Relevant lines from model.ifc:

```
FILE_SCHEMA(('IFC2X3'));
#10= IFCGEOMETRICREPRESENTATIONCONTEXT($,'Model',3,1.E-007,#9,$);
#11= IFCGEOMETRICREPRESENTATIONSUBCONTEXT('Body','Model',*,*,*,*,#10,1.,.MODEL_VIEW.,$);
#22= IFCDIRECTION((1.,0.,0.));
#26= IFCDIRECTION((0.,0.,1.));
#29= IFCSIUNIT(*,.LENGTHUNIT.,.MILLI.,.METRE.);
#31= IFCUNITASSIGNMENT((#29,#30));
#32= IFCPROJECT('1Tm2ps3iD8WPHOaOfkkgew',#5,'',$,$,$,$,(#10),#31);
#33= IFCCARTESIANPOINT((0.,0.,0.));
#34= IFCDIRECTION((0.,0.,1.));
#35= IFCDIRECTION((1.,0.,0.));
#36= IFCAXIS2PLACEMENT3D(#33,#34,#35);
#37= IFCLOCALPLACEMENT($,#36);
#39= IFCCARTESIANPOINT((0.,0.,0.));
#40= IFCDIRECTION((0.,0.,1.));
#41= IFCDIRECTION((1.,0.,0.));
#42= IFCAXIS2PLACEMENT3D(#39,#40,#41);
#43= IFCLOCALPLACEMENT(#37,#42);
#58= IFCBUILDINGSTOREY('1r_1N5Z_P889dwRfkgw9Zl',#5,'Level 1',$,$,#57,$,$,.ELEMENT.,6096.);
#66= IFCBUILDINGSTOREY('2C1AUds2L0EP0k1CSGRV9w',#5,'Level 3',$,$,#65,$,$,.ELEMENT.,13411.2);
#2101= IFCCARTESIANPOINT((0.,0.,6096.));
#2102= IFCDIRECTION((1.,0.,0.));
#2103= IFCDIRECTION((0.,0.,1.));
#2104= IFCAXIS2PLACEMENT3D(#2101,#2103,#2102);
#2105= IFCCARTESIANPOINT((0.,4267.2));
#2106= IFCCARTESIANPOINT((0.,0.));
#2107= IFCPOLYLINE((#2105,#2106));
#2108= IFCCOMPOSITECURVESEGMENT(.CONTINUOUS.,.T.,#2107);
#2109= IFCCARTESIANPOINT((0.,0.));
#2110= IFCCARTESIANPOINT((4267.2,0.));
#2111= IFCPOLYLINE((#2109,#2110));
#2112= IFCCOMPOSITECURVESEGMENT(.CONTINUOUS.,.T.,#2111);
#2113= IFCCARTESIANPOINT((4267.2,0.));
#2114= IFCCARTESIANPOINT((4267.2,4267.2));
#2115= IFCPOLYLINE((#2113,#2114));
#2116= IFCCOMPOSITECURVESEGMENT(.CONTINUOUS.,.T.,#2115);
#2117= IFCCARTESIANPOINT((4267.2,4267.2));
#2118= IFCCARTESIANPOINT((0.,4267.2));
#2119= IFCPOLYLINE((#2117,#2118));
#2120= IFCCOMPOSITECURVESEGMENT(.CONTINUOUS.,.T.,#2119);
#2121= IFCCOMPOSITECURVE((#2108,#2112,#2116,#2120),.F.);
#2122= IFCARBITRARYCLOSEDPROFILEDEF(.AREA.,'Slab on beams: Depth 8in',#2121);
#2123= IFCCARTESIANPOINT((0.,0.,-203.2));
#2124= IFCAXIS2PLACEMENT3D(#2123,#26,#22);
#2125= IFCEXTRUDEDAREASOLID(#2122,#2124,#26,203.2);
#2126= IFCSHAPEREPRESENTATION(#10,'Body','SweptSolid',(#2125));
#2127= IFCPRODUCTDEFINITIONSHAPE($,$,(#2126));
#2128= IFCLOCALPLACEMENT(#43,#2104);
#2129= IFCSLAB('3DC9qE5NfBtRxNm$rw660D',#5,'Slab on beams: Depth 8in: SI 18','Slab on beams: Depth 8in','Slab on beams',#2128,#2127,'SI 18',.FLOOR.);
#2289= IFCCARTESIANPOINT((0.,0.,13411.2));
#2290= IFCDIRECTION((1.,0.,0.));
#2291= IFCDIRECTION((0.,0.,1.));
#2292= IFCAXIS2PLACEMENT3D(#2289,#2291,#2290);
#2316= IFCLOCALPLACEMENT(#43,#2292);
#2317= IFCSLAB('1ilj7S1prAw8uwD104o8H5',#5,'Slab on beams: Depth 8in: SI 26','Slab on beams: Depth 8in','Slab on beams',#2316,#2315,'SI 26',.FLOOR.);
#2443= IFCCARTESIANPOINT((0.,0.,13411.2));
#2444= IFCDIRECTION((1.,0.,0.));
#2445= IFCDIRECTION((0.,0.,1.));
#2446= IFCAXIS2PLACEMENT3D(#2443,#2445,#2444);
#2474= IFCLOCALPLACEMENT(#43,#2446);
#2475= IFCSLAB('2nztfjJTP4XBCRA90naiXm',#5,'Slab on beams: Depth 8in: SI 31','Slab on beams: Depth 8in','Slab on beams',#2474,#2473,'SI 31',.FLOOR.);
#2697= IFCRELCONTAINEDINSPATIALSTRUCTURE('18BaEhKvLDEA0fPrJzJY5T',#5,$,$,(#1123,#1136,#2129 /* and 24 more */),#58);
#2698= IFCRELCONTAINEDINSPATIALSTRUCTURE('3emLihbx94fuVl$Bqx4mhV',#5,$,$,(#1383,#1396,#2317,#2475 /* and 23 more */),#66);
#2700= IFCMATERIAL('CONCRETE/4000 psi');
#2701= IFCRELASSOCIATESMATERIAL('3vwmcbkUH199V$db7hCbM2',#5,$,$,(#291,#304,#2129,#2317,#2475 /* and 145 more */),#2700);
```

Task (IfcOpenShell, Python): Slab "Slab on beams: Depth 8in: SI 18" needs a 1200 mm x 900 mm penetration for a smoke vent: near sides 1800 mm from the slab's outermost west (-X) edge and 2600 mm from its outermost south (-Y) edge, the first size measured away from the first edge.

```python
import numpy as np
import ifcopenshell
import ifcopenshell.api.feature
import ifcopenshell.api.geometry
import ifcopenshell.api.root
import ifcopenshell.geom
import ifcopenshell.util.placement
import ifcopenshell.util.representation
import ifcopenshell.util.shape
import ifcopenshell.util.unit

model = ifcopenshell.open("model.ifc")
unit_scale = ifcopenshell.util.unit.calculate_unit_scale(model)
settings = ifcopenshell.geom.settings()


def volume(element):
    """Net volume in cubic metres, openings subtracted."""
    shape = ifcopenshell.geom.create_shape(settings, element)
    return ifcopenshell.util.shape.get_volume(shape.geometry)


slab = model.by_id(2129)
before = volume(slab)

# Extent in the slab's own axes, in metres. The edges named are its -X and -Y sides.
slab_shape = ifcopenshell.geom.create_shape(settings, slab)
vertices = ifcopenshell.util.shape.get_vertices(slab_shape.geometry)
x_min, y_min, bottom = vertices.min(axis=0)
top = vertices[:, 2].max()

opening = ifcopenshell.api.root.create_entity(model, ifc_class="IfcOpeningElement", name="Smoke vent opening")
context = ifcopenshell.util.representation.get_context(model, "Model", "Body", "MODEL_VIEW")
width, depth = 1.2, 0.9
outline = [(0.0, 0.0), (width, 0.0), (width, depth), (0.0, depth), (0.0, 0.0)]
# Overshoot both faces by 50 mm so the cut is clean.
shape = ifcopenshell.api.geometry.add_slab_representation(
    model, context=context, depth=top - bottom + 0.1, polyline=outline
)
ifcopenshell.api.geometry.assign_representation(model, product=opening, representation=shape)

matrix = ifcopenshell.util.placement.get_local_placement(slab.ObjectPlacement)
matrix[:, 3] = matrix @ np.append(np.array([x_min + 1.8, y_min + 2.6, bottom - 0.05]) / unit_scale, 1.0)
ifcopenshell.api.geometry.edit_object_placement(model, product=opening, matrix=matrix, is_si=False)
ifcopenshell.api.feature.add_feature(model, feature=opening, element=slab)

after = volume(slab)

print(f"slab volume {before:.3f} -> {after:.3f} m3")

model.write("model-out.ifc")
```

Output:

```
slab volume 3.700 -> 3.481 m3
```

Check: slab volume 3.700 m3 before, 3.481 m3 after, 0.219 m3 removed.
